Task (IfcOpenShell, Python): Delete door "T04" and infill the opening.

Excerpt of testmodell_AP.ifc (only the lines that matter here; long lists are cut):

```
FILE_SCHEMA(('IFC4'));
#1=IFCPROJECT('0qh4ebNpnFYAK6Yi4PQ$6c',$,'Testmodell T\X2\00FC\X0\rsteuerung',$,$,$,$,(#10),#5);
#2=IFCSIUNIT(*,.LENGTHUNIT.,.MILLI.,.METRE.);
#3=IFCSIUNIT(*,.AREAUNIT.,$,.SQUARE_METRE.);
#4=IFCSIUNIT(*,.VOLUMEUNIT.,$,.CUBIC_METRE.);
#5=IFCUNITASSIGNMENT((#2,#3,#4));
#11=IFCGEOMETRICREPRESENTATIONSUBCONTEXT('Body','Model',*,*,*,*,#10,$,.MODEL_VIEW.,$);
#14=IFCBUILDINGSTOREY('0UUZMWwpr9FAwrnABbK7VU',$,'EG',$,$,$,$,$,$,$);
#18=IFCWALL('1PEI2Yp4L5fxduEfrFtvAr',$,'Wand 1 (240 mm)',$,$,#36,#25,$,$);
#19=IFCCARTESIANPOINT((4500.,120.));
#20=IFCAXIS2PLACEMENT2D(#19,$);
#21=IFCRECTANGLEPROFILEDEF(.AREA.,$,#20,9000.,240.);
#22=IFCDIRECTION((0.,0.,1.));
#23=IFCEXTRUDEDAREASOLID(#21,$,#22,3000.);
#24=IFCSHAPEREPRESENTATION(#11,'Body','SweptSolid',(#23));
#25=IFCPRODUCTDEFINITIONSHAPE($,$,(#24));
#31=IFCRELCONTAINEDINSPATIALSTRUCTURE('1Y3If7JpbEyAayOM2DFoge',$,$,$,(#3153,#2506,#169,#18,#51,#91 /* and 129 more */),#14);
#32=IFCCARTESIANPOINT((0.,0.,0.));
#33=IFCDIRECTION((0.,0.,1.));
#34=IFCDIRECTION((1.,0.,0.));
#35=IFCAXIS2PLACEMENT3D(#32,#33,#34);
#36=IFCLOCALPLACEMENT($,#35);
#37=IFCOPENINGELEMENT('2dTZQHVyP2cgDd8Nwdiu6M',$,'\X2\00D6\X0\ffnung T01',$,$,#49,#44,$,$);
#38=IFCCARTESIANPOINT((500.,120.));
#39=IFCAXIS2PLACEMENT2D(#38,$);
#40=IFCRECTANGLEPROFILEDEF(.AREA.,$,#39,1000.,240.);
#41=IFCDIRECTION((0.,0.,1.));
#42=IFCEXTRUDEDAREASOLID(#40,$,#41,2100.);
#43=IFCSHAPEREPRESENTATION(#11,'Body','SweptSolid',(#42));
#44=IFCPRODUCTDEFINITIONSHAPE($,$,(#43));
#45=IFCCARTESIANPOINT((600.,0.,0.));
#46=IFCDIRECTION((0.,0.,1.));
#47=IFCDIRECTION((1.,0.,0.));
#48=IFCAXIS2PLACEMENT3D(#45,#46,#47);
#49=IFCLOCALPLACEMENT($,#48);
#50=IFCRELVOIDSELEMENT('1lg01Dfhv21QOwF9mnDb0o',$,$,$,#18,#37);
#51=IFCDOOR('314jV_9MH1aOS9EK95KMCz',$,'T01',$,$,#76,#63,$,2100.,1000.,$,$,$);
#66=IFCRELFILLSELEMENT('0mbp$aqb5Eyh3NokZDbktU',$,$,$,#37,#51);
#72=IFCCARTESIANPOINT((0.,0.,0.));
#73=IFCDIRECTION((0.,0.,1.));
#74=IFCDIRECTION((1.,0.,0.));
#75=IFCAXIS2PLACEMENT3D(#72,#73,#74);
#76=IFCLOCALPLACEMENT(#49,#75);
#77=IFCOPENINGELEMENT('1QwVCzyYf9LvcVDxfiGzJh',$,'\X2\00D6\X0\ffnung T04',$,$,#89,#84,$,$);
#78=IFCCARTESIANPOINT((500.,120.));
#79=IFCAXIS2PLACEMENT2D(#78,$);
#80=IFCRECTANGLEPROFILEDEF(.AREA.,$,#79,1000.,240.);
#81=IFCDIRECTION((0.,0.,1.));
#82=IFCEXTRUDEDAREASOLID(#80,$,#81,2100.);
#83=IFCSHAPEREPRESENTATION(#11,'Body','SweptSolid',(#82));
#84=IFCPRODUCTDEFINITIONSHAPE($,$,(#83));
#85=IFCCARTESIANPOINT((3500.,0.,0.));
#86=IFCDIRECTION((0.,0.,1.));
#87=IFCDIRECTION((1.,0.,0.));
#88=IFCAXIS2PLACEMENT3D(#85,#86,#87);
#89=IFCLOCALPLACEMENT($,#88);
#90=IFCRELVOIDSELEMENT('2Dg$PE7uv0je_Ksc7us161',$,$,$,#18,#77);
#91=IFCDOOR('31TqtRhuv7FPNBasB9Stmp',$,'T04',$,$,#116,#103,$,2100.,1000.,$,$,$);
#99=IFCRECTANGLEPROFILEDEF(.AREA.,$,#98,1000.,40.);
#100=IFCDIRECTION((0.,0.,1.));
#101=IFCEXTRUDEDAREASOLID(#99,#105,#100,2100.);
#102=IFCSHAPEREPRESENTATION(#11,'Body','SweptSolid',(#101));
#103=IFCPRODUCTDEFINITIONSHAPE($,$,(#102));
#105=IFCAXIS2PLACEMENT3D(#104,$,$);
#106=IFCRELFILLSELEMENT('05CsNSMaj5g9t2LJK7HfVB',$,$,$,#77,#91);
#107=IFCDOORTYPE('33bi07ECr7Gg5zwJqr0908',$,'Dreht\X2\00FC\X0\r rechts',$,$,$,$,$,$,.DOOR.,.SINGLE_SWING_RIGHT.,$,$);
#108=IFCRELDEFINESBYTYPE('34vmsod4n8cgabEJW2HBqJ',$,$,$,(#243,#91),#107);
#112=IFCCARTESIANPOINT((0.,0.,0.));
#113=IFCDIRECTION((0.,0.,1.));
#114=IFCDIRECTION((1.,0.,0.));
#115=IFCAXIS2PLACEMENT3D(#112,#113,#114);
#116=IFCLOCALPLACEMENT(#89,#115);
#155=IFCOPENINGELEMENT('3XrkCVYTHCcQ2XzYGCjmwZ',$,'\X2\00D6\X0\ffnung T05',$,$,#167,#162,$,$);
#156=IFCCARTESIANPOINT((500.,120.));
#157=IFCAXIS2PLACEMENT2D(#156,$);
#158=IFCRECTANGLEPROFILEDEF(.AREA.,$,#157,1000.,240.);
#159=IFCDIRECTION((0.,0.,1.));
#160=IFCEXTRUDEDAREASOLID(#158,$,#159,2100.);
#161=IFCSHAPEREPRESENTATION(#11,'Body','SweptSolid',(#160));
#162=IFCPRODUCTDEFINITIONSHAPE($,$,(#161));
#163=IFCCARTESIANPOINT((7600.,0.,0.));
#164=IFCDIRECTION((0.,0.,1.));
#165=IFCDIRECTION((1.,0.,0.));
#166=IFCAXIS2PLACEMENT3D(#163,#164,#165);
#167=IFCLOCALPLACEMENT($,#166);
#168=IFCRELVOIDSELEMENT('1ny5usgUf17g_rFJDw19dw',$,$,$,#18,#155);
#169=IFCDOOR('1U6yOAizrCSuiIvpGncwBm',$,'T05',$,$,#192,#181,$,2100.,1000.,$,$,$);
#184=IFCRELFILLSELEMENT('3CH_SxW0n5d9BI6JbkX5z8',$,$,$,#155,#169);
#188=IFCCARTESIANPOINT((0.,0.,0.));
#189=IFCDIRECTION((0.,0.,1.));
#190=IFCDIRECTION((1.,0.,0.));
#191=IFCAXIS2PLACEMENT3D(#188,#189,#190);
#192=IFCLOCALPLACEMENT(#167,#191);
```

```python
import ifcopenshell
import ifcopenshell.api.feature
import ifcopenshell.api.root
import ifcopenshell.geom
import ifcopenshell.util.shape

model = ifcopenshell.open("testmodell_AP.ifc")
settings = ifcopenshell.geom.settings()


def volume(element):
    """Net volume in cubic metres, openings subtracted."""
    shape = ifcopenshell.geom.create_shape(settings, element)
    return ifcopenshell.util.shape.get_volume(shape.geometry)


door = model.by_guid("31TqtRhuv7FPNBasB9Stmp")
opening = door.FillsVoids[0].RelatingOpeningElement
wall = opening.VoidsElements[0].RelatingBuildingElement
before = volume(wall)

ifcopenshell.api.root.remove_product(model, product=door)
ifcopenshell.api.feature.remove_feature(model, feature=opening)

after = volume(wall)

print(f"wall volume {before:.3f} -> {after:.3f} m3")

model.write("testmodell_AP_v2.ifc")
```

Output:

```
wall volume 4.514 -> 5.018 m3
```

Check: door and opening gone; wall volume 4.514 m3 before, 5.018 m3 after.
